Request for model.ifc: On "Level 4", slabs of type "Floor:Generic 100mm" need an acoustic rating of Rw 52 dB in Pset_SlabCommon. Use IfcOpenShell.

First a look at what the model holds.

```python
import ifcopenshell
import ifcopenshell.util.element

model = ifcopenshell.open("model.ifc")
print(model.schema)
storey = next(s for s in model.by_type("IfcBuildingStorey") if s.Name == "Level 4")
slabs = [e for e in ifcopenshell.util.element.get_decomposition(storey) if e.is_a("IfcSlab")]
seen = {}
for e in slabs:
    element_type = ifcopenshell.util.element.get_type(e)
    key = (element_type.Name if element_type != e and element_type else None, ifcopenshell.util.element.get_pset(e, "Pset_SlabCommon", "AcousticRating"))
    seen[key] = seen.get(key, 0) + 1
for (name, value), count in sorted(seen.items(), key=str):
    print(count, "x", name, "|", value)
```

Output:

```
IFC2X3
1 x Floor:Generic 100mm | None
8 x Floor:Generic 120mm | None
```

```python
import ifcopenshell
import ifcopenshell.api.pset
import ifcopenshell.util.element

model = ifcopenshell.open("model.ifc")

storey = next(s for s in model.by_type("IfcBuildingStorey") if s.Name == "Level 4")
slabs = [e for e in ifcopenshell.util.element.get_decomposition(storey) if e.is_a("IfcSlab")]

count = 0
for e in slabs:
    element_type = ifcopenshell.util.element.get_type(e)
    if element_type in (None, e) or element_type.Name != "Floor:Generic 100mm":
        continue
    # add_pset returns the element's existing set when there is one.
    pset = ifcopenshell.api.pset.add_pset(model, product=e, name="Pset_SlabCommon")
    ifcopenshell.api.pset.edit_pset(model, pset=pset, properties={"AcousticRating": "Rw 52 dB"})
    count += 1

print(count, "slabs updated")

model.write("model-out.ifc")
```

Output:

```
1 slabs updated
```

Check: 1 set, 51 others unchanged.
